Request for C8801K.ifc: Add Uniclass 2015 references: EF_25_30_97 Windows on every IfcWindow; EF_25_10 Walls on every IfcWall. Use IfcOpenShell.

First a look at what the model holds.

```python
import ifcopenshell

model = ifcopenshell.open("C8801K.ifc")
print(model.schema)
print("classifications:", [c.Name for c in model.by_type("IfcClassification")])
for ifc_class in ("IfcDoor", "IfcRoof", "IfcStair", "IfcWall", "IfcWindow"):
    print(ifc_class, len(model.by_type(ifc_class)))
```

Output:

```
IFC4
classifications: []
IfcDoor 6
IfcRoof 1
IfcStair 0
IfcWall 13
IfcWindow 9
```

```python
import ifcopenshell
import ifcopenshell.api.classification

model = ifcopenshell.open("C8801K.ifc")

system = ifcopenshell.api.classification.add_classification(model, classification="Uniclass 2015")

codes = {
    "IfcWindow": ("EF_25_30_97", "Windows"),
    "IfcWall": ("EF_25_10", "Walls"),
}
for ifc_class, (code, name) in codes.items():
    products = model.by_type(ifc_class)
    ifcopenshell.api.classification.add_reference(
        model, products=products, classification=system, identification=code, name=name
    )
    print(code, len(products))

model.write("C8801K_edited.ifc")
```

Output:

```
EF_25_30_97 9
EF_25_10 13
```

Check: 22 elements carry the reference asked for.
